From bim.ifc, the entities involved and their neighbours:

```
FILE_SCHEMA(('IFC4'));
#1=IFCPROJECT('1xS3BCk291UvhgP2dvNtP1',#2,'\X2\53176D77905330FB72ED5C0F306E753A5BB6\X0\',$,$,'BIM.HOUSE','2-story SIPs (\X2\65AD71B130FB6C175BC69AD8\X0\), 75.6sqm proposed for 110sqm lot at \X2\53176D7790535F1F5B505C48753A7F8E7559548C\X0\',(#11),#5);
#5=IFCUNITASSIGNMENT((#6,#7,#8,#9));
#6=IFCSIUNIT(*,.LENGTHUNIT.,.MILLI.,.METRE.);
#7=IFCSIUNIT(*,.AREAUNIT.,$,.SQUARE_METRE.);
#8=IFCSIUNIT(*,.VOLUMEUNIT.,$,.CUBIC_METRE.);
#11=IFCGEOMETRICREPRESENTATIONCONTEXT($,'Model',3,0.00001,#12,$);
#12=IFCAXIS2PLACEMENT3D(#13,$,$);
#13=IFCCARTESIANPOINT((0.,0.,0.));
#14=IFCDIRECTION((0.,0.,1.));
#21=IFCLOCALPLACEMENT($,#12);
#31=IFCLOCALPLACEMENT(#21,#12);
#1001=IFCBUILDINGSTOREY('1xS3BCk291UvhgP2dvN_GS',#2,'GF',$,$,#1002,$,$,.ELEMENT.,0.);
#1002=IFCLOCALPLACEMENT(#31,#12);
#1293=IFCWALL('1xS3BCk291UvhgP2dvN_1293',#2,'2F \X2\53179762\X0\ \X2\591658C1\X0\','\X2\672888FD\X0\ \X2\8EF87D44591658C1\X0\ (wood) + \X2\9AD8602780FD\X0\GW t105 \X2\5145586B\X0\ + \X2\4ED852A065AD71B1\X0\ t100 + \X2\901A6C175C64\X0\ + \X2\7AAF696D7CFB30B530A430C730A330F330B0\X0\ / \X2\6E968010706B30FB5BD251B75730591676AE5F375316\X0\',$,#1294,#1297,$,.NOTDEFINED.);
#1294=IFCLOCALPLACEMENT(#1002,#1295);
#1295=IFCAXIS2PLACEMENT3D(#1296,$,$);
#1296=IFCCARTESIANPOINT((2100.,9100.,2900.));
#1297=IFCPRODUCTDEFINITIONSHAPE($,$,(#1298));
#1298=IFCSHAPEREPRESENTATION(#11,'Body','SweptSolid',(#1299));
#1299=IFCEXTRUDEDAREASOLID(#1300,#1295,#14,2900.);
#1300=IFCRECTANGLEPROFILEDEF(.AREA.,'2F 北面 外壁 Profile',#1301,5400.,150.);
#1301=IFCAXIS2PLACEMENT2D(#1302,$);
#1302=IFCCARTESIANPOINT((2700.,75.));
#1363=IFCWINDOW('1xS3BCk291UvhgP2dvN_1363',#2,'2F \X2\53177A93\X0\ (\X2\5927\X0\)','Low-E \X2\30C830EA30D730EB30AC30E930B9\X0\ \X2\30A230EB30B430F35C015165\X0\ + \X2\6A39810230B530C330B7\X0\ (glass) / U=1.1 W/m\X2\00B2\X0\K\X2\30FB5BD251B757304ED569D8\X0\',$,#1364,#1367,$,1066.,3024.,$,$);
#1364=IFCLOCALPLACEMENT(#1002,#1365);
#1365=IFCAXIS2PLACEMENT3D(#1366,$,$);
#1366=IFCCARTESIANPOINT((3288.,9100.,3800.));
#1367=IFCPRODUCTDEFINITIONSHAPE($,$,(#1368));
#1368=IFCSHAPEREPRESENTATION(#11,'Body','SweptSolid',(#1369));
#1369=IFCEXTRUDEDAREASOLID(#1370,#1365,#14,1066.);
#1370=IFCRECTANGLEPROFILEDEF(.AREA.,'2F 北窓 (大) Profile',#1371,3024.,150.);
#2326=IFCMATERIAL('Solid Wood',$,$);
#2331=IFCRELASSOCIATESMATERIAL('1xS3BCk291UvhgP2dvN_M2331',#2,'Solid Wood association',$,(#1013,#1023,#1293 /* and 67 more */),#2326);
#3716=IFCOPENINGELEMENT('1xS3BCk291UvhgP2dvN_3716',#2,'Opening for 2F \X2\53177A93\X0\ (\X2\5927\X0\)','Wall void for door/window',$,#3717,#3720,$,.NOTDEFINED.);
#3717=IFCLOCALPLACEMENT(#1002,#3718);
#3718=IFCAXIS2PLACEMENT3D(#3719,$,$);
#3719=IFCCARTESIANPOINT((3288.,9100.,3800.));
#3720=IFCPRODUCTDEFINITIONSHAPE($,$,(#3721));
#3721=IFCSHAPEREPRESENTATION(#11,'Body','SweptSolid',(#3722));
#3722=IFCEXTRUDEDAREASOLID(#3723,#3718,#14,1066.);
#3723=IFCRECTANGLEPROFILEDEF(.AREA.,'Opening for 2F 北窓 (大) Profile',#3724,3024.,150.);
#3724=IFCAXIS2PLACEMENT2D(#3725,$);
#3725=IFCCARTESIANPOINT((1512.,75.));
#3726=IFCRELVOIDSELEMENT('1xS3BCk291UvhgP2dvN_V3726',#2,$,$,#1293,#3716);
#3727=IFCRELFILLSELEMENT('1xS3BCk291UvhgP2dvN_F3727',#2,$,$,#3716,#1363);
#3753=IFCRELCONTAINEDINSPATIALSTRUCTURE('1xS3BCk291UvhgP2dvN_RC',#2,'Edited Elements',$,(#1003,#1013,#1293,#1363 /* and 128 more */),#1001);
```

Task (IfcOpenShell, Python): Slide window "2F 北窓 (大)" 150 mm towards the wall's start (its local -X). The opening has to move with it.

```python
import ifcopenshell
import ifcopenshell.api.geometry
import ifcopenshell.util.placement
import ifcopenshell.util.unit

model = ifcopenshell.open("bim.ifc")
unit_scale = ifcopenshell.util.unit.calculate_unit_scale(model)

window = model.by_id(1363)
opening = window.FillsVoids[0].RelatingOpeningElement
wall = opening.VoidsElements[0].RelatingBuildingElement

wall_matrix = ifcopenshell.util.placement.get_local_placement(wall.ObjectPlacement)
shift = wall_matrix[:3, 0] * -0.15 / unit_scale
before = ifcopenshell.util.placement.get_local_placement(window.ObjectPlacement)[:3, 3].copy()

# The window is not placed relative to its opening, so move both.
for product in (opening, window):
    matrix = ifcopenshell.util.placement.get_local_placement(product.ObjectPlacement)
    matrix[:3, 3] += shift
    ifcopenshell.api.geometry.edit_object_placement(model, product=product, matrix=matrix, is_si=False)

after = ifcopenshell.util.placement.get_local_placement(window.ObjectPlacement)[:3, 3]
print("window moved by", (after - before).round(3) + 0.0)

model.write("bim_updated.ifc")
```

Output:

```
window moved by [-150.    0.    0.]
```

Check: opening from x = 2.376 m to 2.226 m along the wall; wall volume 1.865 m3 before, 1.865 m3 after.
